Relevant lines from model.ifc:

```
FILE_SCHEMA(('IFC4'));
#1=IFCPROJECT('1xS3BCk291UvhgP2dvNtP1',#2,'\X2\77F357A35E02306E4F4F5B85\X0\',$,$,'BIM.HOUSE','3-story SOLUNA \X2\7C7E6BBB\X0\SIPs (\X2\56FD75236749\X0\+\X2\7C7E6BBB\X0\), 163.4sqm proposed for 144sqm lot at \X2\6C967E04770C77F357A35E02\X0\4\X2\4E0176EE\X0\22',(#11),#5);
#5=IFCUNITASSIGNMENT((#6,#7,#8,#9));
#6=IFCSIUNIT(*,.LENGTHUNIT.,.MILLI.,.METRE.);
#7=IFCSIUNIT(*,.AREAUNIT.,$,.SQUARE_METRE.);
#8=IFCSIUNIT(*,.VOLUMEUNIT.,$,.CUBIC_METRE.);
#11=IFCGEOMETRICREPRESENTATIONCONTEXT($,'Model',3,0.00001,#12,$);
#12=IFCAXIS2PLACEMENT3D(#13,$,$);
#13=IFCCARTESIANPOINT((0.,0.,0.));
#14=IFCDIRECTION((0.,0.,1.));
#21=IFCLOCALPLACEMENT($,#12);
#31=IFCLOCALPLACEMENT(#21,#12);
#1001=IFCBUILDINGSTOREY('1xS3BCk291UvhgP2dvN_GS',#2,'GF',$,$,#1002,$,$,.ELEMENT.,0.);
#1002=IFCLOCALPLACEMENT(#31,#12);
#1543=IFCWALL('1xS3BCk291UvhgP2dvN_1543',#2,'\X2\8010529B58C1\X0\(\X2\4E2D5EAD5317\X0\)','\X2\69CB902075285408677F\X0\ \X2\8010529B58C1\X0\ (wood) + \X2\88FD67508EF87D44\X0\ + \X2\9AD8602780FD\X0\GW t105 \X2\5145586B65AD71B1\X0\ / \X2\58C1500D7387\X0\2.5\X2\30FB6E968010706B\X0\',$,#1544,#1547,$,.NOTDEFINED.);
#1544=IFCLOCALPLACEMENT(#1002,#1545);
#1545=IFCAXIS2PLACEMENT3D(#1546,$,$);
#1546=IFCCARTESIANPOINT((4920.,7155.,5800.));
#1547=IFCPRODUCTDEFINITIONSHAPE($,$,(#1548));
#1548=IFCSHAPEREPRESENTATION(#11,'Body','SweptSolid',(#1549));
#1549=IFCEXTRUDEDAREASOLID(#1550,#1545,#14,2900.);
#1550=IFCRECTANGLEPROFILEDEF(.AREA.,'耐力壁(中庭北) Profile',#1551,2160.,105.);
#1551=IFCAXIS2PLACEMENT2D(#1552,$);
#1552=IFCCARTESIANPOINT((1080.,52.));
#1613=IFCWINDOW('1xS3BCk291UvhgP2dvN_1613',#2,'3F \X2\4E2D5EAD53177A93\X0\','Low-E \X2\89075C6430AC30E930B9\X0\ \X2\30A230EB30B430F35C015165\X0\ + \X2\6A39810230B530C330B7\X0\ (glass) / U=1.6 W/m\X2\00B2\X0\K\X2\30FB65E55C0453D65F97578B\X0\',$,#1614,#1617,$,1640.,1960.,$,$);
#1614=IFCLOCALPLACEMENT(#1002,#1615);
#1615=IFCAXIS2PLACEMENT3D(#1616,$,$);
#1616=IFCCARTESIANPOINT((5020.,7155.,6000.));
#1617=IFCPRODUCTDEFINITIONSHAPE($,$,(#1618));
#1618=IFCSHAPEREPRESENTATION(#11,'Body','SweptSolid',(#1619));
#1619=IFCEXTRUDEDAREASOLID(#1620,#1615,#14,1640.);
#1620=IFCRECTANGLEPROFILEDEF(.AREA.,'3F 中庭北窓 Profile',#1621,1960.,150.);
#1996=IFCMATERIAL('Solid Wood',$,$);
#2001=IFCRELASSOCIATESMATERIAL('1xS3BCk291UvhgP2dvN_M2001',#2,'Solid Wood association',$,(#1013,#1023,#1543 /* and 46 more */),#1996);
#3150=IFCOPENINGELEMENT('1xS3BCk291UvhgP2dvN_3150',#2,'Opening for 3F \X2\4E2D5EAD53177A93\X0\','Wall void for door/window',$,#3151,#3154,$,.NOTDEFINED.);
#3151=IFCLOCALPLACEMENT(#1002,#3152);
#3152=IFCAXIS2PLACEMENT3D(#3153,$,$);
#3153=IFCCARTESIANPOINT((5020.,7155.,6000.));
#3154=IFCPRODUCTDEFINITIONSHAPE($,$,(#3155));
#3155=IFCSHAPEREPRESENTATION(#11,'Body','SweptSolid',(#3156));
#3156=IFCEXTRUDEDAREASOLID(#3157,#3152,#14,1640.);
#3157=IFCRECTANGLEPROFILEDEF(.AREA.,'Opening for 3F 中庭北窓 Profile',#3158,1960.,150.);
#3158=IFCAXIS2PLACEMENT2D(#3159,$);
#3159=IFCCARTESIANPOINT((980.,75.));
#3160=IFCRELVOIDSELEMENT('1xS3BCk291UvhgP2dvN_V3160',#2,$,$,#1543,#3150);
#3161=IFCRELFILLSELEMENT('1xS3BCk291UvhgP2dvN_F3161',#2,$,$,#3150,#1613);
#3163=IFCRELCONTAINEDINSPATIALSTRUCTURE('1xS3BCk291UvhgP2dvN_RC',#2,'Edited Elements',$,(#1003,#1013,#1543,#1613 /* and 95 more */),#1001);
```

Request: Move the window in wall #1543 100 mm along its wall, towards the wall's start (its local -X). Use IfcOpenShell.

```python
import ifcopenshell
import ifcopenshell.api.geometry
import ifcopenshell.util.placement
import ifcopenshell.util.unit

model = ifcopenshell.open("model.ifc")
unit_scale = ifcopenshell.util.unit.calculate_unit_scale(model)

window = model.by_guid("1xS3BCk291UvhgP2dvN_1613")
opening = window.FillsVoids[0].RelatingOpeningElement
wall = opening.VoidsElements[0].RelatingBuildingElement

wall_matrix = ifcopenshell.util.placement.get_local_placement(wall.ObjectPlacement)
shift = wall_matrix[:3, 0] * -0.1 / unit_scale
before = ifcopenshell.util.placement.get_local_placement(window.ObjectPlacement)[:3, 3].copy()

# The window is not placed relative to its opening, so move both.
for product in (opening, window):
    matrix = ifcopenshell.util.placement.get_local_placement(product.ObjectPlacement)
    matrix[:3, 3] += shift
    ifcopenshell.api.geometry.edit_object_placement(model, product=product, matrix=matrix, is_si=False)

after = ifcopenshell.util.placement.get_local_placement(window.ObjectPlacement)[:3, 3]
print("window moved by", (after - before).round(3) + 0.0)

model.write("model_rev.ifc")
```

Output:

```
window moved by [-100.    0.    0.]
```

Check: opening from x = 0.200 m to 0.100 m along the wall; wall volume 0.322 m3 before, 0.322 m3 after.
